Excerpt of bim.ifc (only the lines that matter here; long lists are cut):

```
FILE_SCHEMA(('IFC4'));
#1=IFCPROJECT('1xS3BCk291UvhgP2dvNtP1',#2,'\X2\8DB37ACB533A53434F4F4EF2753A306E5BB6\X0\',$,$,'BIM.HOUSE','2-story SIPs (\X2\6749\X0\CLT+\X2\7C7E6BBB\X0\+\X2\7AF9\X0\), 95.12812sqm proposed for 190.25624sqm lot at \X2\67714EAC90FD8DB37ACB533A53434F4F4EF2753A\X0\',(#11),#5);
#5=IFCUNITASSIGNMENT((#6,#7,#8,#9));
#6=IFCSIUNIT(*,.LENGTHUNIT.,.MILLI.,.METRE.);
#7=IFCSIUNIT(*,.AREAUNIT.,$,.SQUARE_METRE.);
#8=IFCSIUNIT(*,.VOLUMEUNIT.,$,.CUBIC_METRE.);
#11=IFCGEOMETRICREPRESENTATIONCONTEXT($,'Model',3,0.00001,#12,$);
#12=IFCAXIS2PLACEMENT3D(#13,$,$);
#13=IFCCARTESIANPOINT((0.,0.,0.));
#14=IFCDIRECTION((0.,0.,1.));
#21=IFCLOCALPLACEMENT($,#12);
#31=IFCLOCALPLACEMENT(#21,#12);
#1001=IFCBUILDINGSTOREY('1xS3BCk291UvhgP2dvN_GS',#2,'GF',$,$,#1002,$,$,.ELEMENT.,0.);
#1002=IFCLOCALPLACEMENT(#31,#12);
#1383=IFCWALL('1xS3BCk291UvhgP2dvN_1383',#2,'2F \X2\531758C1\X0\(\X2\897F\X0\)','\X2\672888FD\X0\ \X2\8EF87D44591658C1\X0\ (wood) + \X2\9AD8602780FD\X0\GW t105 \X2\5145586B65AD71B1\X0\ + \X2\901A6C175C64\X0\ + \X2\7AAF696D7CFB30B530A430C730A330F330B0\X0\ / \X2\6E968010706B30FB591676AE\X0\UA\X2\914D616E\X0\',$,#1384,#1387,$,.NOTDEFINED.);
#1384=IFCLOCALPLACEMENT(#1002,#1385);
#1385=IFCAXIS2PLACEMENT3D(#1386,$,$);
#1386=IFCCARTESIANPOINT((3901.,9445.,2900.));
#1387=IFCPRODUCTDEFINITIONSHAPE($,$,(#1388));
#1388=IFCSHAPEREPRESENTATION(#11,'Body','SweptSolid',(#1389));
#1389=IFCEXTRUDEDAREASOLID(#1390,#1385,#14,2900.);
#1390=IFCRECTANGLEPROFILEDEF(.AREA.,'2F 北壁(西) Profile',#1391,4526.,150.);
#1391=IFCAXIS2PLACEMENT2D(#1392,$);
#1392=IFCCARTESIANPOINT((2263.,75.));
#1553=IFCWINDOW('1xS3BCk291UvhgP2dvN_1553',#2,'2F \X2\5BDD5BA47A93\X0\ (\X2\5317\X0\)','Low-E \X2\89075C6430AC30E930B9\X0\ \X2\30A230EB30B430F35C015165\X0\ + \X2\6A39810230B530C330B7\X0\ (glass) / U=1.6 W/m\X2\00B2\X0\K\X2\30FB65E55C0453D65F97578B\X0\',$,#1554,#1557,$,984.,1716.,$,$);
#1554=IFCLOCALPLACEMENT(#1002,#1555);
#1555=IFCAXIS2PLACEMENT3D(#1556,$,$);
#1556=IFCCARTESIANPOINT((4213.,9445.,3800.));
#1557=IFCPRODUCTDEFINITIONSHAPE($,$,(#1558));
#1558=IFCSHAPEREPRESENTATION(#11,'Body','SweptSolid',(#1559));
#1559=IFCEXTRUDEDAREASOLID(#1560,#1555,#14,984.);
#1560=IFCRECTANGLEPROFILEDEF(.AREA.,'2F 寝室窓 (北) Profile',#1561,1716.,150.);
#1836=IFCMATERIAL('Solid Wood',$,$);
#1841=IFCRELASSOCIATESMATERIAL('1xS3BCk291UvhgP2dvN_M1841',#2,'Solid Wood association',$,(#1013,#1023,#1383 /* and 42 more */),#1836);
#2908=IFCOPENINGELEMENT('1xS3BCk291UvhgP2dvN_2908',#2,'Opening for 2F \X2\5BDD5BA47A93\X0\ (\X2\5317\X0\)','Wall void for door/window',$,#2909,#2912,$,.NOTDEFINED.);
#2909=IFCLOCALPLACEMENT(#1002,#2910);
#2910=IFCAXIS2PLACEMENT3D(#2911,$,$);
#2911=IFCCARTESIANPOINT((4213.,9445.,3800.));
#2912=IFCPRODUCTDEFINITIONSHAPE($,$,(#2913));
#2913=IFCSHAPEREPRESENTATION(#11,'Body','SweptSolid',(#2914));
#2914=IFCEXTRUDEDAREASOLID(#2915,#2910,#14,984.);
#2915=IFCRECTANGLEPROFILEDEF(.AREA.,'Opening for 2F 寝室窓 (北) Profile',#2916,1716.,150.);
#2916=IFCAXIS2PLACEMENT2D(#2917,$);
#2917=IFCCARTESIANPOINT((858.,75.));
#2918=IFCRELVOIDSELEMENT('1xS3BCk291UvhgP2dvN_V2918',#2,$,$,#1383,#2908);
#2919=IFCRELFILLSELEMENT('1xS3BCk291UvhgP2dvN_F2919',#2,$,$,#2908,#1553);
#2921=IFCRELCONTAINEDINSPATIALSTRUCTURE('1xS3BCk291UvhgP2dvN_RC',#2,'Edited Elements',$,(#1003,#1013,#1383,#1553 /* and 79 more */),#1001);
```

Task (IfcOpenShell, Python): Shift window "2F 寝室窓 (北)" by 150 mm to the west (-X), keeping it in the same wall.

```python
import ifcopenshell
import ifcopenshell.api.geometry
import ifcopenshell.util.placement

model = ifcopenshell.open("bim.ifc")

window = model.by_id(1553)
opening = window.FillsVoids[0].RelatingOpeningElement
wall = opening.VoidsElements[0].RelatingBuildingElement

wall_matrix = ifcopenshell.util.placement.get_local_placement(wall.ObjectPlacement)
shift = wall_matrix[:3, 0] * -150.0
before = ifcopenshell.util.placement.get_local_placement(window.ObjectPlacement)[:3, 3].copy()

# The window is not placed relative to its opening, so move both.
for product in (opening, window):
    matrix = ifcopenshell.util.placement.get_local_placement(product.ObjectPlacement)
    matrix[:3, 3] += shift
    ifcopenshell.api.geometry.edit_object_placement(model, product=product, matrix=matrix, is_si=False)

after = ifcopenshell.util.placement.get_local_placement(window.ObjectPlacement)[:3, 3]
print("window moved by", (after - before).round(3) + 0.0)

model.write("bim_edited.ifc")
```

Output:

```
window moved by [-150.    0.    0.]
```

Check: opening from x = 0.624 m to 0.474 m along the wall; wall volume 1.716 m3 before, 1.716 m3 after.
